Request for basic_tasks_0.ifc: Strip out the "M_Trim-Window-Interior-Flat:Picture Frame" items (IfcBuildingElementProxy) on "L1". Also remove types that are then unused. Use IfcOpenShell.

First a look at what the model holds.

```python
import ifcopenshell
import ifcopenshell.util.element

model = ifcopenshell.open("basic_tasks_0.ifc")
print(model.schema)
storey = next(s for s in model.by_type("IfcBuildingStorey") if s.Name == "L1")
proxies = [e for e in ifcopenshell.util.element.get_decomposition(storey) if e.is_a("IfcBuildingElementProxy")]
seen = {}
for e in proxies:
    element_type = ifcopenshell.util.element.get_type(e)
    name = element_type.Name if element_type not in (None, e) else None
    seen[name] = seen.get(name, 0) + 1
for name, count in sorted(seen.items(), key=str):
    print(count, "x", name)
```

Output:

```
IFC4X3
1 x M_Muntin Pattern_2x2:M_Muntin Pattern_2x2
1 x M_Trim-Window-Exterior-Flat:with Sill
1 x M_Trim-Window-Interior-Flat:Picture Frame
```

```python
import ifcopenshell
import ifcopenshell.api.root
import ifcopenshell.util.element

model = ifcopenshell.open("basic_tasks_0.ifc")

storey = next(s for s in model.by_type("IfcBuildingStorey") if s.Name == "L1")
proxies = [e for e in ifcopenshell.util.element.get_decomposition(storey) if e.is_a("IfcBuildingElementProxy")]
targets = [e for e in proxies if (t := ifcopenshell.util.element.get_type(e)) not in (None, e) and t.Name == "M_Trim-Window-Interior-Flat:Picture Frame"]
types = {ifcopenshell.util.element.get_type(e) for e in targets} - {None, *targets}

for e in targets:
    ifcopenshell.api.root.remove_product(model, product=e)
print(len(targets), "removed")

unused = [t for t in types if not ifcopenshell.util.element.get_types(t)]
for t in unused:
    ifcopenshell.api.root.remove_product(model, product=t)
print(len(unused), "unused types removed")

model.write("basic_tasks_0_v2.ifc")
```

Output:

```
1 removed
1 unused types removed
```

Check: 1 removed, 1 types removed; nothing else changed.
